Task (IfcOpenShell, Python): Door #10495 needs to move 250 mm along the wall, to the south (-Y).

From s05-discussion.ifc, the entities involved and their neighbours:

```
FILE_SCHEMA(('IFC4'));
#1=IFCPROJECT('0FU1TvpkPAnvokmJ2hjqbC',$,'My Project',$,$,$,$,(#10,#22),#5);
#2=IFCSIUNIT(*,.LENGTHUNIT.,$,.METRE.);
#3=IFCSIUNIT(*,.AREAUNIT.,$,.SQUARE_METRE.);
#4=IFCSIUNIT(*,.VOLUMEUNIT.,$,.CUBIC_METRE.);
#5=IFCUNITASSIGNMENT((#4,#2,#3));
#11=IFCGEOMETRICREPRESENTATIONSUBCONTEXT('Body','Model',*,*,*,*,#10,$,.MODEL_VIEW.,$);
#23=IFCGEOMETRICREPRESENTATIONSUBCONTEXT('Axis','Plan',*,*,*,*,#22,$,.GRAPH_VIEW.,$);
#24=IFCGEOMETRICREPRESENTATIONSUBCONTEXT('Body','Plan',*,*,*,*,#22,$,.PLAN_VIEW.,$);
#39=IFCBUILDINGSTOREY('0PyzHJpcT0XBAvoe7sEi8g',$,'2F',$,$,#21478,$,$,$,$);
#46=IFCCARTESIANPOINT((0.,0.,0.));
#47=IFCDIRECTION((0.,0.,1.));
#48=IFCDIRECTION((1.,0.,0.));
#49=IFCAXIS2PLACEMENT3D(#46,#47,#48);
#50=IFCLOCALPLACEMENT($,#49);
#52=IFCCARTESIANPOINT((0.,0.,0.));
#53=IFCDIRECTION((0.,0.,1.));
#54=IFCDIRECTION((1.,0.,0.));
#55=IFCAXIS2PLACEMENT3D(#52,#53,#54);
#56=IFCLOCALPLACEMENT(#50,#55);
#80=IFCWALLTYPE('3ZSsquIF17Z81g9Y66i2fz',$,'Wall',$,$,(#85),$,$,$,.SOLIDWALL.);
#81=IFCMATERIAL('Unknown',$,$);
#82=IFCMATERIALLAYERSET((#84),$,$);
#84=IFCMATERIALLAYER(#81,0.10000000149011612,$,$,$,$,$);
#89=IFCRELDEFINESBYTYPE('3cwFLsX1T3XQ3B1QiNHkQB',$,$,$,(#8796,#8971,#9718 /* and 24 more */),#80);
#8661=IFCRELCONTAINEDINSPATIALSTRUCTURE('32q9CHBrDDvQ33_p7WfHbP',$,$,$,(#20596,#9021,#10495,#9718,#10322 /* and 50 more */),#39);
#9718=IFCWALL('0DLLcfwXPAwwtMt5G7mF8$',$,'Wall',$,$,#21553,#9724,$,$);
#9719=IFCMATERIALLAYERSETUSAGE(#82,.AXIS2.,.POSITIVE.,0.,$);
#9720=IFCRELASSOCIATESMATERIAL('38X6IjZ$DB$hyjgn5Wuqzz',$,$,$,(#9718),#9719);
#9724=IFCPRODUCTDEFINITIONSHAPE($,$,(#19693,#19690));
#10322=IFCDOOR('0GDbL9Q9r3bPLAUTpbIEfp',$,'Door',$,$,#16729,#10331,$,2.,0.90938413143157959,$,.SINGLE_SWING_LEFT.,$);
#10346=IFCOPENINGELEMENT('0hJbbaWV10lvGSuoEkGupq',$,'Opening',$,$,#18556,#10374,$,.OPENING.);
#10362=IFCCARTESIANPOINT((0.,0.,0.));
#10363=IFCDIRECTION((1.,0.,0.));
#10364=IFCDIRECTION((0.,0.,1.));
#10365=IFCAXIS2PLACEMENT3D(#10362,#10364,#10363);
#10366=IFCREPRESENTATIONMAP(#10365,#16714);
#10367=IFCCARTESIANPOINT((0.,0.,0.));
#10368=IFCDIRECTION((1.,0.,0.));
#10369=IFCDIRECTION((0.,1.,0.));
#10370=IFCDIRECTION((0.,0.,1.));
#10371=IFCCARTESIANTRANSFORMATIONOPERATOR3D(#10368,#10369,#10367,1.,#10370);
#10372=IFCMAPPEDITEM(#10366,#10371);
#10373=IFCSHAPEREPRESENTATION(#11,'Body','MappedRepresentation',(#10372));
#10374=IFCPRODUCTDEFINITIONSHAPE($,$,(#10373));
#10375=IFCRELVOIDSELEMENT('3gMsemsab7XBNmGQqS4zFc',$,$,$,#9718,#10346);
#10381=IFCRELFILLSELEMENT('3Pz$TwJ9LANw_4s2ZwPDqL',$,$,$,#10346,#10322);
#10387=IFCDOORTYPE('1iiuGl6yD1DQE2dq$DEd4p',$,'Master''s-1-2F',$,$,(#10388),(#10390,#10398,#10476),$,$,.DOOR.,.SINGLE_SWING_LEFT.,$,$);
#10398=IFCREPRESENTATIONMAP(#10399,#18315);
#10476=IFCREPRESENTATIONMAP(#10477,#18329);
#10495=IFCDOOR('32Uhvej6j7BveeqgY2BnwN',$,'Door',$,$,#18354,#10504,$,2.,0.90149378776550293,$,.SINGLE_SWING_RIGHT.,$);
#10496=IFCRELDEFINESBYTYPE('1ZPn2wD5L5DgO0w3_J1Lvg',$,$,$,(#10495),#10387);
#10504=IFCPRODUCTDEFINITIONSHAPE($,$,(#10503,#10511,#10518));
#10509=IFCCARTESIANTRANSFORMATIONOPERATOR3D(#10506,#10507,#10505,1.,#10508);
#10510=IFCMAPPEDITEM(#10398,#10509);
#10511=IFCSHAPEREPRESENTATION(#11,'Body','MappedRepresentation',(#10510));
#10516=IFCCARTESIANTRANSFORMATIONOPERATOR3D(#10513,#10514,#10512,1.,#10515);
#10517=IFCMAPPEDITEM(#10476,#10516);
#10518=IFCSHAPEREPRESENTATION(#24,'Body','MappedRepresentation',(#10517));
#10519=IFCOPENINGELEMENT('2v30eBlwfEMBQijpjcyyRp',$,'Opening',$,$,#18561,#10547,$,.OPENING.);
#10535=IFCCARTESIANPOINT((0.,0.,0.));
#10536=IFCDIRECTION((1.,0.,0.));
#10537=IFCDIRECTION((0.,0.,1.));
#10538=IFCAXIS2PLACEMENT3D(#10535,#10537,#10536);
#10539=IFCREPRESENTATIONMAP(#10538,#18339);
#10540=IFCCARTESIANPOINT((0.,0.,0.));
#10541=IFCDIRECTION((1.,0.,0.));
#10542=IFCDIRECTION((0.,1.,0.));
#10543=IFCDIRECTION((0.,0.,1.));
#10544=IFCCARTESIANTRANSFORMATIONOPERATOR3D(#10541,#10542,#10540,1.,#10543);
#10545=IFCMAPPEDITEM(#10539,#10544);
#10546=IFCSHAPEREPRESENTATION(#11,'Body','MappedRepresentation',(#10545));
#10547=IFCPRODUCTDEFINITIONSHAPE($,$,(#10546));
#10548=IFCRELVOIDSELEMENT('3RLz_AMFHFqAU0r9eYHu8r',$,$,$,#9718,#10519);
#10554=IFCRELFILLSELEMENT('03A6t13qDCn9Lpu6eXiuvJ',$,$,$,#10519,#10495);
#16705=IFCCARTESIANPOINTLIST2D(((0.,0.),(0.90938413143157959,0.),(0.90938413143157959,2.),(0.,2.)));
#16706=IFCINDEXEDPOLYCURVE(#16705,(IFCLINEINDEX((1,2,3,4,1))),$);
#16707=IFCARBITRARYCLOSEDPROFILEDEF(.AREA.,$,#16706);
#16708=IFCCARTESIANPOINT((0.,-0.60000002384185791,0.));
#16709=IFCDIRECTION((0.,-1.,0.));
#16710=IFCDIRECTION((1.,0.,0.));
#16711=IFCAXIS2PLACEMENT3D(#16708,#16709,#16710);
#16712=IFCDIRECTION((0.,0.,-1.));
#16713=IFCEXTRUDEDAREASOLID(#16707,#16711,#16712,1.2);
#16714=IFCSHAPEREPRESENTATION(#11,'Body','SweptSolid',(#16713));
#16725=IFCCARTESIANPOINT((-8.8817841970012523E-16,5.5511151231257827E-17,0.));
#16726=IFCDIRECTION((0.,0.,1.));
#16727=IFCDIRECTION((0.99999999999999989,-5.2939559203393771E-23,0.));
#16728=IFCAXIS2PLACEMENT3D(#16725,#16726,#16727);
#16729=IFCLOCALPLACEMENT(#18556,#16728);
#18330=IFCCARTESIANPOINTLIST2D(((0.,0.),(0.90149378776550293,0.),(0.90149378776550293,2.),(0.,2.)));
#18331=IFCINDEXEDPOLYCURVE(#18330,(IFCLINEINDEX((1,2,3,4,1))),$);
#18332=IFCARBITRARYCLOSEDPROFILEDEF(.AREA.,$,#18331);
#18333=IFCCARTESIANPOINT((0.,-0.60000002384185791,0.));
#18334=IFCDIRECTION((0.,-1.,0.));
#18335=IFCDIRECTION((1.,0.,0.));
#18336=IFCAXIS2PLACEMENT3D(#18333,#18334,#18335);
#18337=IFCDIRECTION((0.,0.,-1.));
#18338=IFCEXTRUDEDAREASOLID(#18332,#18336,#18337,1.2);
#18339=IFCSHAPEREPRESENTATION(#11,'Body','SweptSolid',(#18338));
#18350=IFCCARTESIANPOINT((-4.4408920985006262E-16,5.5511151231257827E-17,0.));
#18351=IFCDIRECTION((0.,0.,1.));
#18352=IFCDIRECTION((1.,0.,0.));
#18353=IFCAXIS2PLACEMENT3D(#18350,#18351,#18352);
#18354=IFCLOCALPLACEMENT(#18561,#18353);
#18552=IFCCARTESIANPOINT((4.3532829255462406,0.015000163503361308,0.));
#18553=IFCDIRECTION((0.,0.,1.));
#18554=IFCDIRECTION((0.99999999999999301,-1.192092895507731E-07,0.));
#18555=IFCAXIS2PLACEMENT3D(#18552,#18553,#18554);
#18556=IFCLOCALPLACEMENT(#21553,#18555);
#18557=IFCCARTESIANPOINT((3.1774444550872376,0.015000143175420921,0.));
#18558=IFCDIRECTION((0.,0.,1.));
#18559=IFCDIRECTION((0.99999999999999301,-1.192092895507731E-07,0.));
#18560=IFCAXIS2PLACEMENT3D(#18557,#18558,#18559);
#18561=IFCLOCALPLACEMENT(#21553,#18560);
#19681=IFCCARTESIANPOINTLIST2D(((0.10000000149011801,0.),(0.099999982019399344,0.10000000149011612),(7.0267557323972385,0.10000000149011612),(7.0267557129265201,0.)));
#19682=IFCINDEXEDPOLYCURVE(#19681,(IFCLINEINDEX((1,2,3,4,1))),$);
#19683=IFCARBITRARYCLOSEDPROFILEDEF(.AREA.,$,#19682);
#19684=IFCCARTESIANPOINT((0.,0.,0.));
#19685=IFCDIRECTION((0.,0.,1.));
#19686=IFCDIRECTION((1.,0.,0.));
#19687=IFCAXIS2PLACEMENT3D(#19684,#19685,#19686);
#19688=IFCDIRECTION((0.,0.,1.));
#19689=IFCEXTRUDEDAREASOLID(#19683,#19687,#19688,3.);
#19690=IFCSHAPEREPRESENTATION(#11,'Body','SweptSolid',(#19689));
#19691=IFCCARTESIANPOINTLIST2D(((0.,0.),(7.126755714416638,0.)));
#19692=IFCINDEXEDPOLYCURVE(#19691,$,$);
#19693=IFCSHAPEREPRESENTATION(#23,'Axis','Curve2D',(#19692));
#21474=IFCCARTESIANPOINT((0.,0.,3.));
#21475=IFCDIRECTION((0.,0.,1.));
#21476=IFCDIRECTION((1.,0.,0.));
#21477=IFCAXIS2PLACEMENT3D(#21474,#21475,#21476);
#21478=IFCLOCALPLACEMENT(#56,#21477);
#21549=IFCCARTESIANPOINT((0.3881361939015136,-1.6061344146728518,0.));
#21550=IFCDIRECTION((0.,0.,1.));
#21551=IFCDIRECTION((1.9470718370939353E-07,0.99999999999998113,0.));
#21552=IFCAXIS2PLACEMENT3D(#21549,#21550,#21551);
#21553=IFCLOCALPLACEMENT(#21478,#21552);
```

```python
import ifcopenshell
import ifcopenshell.api.geometry
import ifcopenshell.util.placement
import ifcopenshell.util.unit

model = ifcopenshell.open("s05-discussion.ifc")
unit_scale = ifcopenshell.util.unit.calculate_unit_scale(model)

door = model.by_id(10495)
opening = door.FillsVoids[0].RelatingOpeningElement
wall = opening.VoidsElements[0].RelatingBuildingElement

wall_matrix = ifcopenshell.util.placement.get_local_placement(wall.ObjectPlacement)
shift = wall_matrix[:3, 0] * -0.25 / unit_scale
before = ifcopenshell.util.placement.get_local_placement(door.ObjectPlacement)[:3, 3].copy()

# The door is placed relative to its opening, so it follows when the opening moves.
matrix = ifcopenshell.util.placement.get_local_placement(opening.ObjectPlacement)
matrix[:3, 3] += shift
ifcopenshell.api.geometry.edit_object_placement(
    model, product=opening, matrix=matrix, is_si=False, should_transform_children=True
)

after = ifcopenshell.util.placement.get_local_placement(door.ObjectPlacement)[:3, 3]
print("door moved by", (after - before).round(3) + 0.0)

model.write("s05-discussion-out.ifc")
```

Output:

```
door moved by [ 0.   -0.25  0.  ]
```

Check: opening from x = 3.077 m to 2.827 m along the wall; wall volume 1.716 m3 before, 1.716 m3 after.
